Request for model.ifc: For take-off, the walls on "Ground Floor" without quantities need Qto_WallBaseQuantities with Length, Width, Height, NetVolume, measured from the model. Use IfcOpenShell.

First a look at what the model holds.

```python
import ifcopenshell
import ifcopenshell.util.element
import ifcopenshell.util.unit

model = ifcopenshell.open("model.ifc")
print(model.schema)
for unit_type in ("LENGTHUNIT", "AREAUNIT", "VOLUMEUNIT"):
    print(unit_type, ifcopenshell.util.unit.calculate_unit_scale(model, unit_type))
storey = next(s for s in model.by_type("IfcBuildingStorey") if s.Name == "Ground Floor")
walls = [e for e in ifcopenshell.util.element.get_decomposition(storey) if e.is_a("IfcWall")]
for e in sorted(walls, key=lambda e: e.id()):
    print(e.id(), e.is_a(), e.Name, list(ifcopenshell.util.element.get_psets(e, qtos_only=True)), sep=" | ")
```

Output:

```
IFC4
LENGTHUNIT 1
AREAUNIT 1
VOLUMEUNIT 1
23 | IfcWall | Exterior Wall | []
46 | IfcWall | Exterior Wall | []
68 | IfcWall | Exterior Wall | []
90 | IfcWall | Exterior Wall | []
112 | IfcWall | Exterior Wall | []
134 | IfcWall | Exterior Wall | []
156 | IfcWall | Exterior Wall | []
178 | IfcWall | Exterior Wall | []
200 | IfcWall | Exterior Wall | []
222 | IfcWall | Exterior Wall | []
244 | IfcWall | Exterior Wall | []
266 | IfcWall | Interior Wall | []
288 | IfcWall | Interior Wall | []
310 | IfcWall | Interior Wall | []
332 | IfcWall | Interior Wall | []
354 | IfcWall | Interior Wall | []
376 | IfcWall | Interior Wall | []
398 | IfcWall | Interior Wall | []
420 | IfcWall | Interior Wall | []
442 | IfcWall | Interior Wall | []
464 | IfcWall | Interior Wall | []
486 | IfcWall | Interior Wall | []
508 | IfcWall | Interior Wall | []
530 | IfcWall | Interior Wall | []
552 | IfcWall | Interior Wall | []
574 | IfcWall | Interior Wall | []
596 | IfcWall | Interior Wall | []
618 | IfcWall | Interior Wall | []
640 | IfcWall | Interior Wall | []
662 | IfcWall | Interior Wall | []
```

```python
import ifcopenshell
import ifcopenshell.api.pset
import ifcopenshell.geom
import ifcopenshell.util.element
import ifcopenshell.util.shape
import ifcopenshell.util.unit

model = ifcopenshell.open("model.ifc")
unit_scale = ifcopenshell.util.unit.calculate_unit_scale(model)
volume_scale = ifcopenshell.util.unit.calculate_unit_scale(model, "VOLUMEUNIT")
settings = ifcopenshell.geom.settings()

storey = next(s for s in model.by_type("IfcBuildingStorey") if s.Name == "Ground Floor")
walls = [e for e in ifcopenshell.util.element.get_decomposition(storey) if e.is_a("IfcWall")]

for e in sorted(walls, key=lambda e: e.id()):
    if ifcopenshell.util.element.get_psets(e, qtos_only=True, should_inherit=False):
        continue
    # Geometry comes back in metres, in the element's own axes.
    shape = ifcopenshell.geom.create_shape(settings, e)
    values = {
        "Length": ifcopenshell.util.shape.get_x(shape.geometry) / unit_scale,
        "Width": ifcopenshell.util.shape.get_y(shape.geometry) / unit_scale,
        "Height": ifcopenshell.util.shape.get_z(shape.geometry) / unit_scale,
        "NetVolume": ifcopenshell.util.shape.get_volume(shape.geometry) / volume_scale,
    }
    qto = ifcopenshell.api.pset.add_qto(model, product=e, name="Qto_WallBaseQuantities")
    ifcopenshell.api.pset.edit_qto(model, qto=qto, properties=values)
    print(e.id(), {k: round(v, 3) for k, v in values.items()})

model.write("model_edited.ifc")
```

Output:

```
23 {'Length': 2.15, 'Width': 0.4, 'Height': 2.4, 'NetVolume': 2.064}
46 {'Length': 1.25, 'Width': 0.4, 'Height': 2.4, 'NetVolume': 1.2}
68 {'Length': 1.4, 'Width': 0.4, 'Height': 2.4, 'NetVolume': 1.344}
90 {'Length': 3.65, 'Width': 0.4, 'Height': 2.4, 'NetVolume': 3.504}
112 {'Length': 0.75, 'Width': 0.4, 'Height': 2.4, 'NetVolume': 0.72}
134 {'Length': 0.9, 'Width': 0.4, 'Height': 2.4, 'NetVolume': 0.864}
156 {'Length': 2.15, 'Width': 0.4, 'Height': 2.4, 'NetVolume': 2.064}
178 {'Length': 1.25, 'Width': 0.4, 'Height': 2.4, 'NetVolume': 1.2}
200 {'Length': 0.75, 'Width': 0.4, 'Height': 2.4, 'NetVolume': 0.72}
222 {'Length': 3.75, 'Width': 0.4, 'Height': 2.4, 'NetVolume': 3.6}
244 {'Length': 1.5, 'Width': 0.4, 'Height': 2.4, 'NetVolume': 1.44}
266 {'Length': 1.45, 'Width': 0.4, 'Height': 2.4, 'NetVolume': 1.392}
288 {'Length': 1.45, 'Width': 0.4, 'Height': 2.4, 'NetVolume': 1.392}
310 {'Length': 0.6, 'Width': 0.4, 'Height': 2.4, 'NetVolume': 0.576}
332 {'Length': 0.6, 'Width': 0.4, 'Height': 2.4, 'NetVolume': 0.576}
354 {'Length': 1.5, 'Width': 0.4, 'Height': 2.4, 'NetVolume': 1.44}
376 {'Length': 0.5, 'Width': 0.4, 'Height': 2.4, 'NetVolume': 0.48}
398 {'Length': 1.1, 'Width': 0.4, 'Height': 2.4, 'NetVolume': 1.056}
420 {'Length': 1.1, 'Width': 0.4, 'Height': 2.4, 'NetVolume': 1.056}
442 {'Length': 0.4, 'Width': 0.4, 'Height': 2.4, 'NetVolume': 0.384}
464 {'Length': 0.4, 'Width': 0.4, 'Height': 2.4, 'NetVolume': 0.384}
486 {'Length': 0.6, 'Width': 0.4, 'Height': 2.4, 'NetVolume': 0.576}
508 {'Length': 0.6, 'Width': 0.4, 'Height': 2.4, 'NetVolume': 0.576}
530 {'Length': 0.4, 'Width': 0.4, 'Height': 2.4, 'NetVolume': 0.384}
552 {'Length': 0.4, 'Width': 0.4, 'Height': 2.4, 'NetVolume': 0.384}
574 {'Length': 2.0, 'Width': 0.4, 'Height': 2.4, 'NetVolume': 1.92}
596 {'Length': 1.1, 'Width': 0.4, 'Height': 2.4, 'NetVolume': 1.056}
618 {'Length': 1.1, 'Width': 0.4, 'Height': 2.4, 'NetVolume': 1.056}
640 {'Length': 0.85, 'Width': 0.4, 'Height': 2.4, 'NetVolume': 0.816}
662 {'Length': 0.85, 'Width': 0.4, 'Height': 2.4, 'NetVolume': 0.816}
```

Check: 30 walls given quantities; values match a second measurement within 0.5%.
